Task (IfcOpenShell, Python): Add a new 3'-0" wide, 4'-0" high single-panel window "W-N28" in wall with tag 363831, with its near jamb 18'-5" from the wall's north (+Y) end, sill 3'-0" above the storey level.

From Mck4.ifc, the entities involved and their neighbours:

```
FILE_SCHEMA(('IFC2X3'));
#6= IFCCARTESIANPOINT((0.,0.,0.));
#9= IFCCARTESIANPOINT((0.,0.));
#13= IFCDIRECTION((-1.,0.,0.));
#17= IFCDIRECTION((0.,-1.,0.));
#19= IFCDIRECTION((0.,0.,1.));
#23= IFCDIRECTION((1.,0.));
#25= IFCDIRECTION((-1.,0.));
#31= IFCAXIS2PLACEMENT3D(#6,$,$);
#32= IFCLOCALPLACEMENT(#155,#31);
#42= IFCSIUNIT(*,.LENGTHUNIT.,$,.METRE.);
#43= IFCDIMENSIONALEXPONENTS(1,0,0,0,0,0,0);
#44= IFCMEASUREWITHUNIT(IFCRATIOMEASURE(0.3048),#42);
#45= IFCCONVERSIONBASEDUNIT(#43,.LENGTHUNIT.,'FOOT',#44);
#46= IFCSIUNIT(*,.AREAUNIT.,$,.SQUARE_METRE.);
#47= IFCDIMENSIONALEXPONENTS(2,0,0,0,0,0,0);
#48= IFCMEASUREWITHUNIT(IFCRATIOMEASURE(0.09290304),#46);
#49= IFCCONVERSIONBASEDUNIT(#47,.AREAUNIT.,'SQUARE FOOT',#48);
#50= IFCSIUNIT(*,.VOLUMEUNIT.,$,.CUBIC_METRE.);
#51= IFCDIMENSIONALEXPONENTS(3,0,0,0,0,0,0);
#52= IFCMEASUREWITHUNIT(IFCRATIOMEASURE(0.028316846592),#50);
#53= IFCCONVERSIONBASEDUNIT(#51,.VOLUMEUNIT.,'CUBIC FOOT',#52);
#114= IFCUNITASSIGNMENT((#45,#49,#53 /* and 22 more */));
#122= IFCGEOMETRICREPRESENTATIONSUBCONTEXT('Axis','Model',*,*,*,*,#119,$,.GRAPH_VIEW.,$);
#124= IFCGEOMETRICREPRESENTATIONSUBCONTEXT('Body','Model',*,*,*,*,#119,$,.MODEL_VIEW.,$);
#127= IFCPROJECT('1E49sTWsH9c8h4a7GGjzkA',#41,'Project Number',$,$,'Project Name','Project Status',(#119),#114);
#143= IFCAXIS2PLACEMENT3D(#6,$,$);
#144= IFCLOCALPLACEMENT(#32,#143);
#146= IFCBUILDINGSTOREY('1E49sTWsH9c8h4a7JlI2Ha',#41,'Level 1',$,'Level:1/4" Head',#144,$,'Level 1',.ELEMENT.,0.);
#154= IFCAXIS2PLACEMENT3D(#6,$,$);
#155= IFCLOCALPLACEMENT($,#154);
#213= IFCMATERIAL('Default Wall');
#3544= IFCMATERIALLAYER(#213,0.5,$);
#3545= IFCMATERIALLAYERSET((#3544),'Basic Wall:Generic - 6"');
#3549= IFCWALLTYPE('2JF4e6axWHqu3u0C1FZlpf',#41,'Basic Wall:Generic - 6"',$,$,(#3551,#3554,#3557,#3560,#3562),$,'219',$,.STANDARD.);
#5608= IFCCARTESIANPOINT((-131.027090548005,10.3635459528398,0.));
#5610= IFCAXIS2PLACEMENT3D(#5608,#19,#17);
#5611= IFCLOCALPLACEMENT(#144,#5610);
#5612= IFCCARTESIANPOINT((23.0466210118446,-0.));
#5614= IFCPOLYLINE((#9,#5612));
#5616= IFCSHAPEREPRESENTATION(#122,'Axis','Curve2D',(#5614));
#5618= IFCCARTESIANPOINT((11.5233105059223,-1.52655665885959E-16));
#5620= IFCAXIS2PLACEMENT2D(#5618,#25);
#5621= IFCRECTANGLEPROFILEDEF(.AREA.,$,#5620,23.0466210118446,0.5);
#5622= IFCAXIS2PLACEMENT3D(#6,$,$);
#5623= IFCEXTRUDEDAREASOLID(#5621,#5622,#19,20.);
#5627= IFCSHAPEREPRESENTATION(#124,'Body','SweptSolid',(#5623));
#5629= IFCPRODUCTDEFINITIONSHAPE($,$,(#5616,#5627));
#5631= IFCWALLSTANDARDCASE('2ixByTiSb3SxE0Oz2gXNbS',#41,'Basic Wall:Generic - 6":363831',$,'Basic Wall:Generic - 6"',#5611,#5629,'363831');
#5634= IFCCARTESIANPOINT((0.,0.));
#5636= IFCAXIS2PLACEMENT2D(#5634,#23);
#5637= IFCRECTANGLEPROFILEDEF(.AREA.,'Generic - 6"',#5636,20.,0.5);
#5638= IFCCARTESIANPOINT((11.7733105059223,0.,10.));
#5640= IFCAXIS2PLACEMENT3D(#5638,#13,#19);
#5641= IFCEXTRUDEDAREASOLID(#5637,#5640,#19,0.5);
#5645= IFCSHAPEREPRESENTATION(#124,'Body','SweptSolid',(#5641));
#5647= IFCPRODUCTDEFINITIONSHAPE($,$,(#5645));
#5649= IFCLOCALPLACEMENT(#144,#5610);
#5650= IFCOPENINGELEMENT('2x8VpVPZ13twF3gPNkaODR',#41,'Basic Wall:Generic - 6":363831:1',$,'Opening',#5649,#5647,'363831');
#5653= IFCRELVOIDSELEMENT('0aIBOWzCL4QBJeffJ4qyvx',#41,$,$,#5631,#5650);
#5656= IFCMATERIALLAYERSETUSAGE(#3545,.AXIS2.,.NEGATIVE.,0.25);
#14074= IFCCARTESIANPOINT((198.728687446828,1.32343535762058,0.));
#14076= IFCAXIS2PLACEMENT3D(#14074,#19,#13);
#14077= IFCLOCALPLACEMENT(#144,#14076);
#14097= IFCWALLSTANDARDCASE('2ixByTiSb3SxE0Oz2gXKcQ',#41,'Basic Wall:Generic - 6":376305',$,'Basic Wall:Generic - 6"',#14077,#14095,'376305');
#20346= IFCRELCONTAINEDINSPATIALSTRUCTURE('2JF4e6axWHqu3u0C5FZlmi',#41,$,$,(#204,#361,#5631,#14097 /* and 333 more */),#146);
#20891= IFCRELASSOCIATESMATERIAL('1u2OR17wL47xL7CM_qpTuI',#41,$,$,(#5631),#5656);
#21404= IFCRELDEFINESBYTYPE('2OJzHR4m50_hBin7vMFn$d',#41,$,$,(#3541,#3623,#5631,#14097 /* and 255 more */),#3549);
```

```python
import numpy as np
import ifcopenshell
import ifcopenshell.api.feature
import ifcopenshell.api.geometry
import ifcopenshell.api.root
import ifcopenshell.api.spatial
import ifcopenshell.api.type
import ifcopenshell.geom
import ifcopenshell.util.element
import ifcopenshell.util.placement
import ifcopenshell.util.representation
import ifcopenshell.util.shape
import ifcopenshell.util.unit

model = ifcopenshell.open("Mck4.ifc")
unit_scale = ifcopenshell.util.unit.calculate_unit_scale(model)
settings = ifcopenshell.geom.settings()


def volume(element):
    """Net volume in cubic metres, openings subtracted."""
    shape = ifcopenshell.geom.create_shape(settings, element)
    return ifcopenshell.util.shape.get_volume(shape.geometry)


wall = model.by_id(5631)
storey = ifcopenshell.util.element.get_container(wall, ifc_class="IfcBuildingStorey")
context = ifcopenshell.util.representation.get_context(model, "Model", "Body", "MODEL_VIEW")
before = volume(wall)

width, height, from_end, sill = 0.9144, 1.2192, 5.6134, 0.9144  # metres

# The wall runs along its own X axis, and the end named is its -X end.
wall_shape = ifcopenshell.geom.create_shape(settings, wall)
x, y, z = ifcopenshell.util.shape.get_vertices(wall_shape.geometry).T
start = x.min() + from_end
face, thickness = float(y.min()), float(y.max() - y.min())
wall_matrix = ifcopenshell.util.placement.get_local_placement(wall.ObjectPlacement)
level = ifcopenshell.util.placement.get_local_placement(storey.ObjectPlacement)[2, 3]


def in_wall(x, y):
    """Placement at x, y metres in the wall's axes, at sill height."""
    matrix = wall_matrix.copy()
    matrix[:, 3] = wall_matrix @ np.array([x / unit_scale, y / unit_scale, 0.0, 1.0])
    matrix[2, 3] = level + sill / unit_scale
    return matrix


# Opening: a box that overshoots both wall faces by 50 mm.
opening = ifcopenshell.api.root.create_entity(model, ifc_class="IfcOpeningElement")
box = ifcopenshell.api.geometry.add_wall_representation(
    model, context=context, length=width, height=height, thickness=thickness + 0.1
)
ifcopenshell.api.geometry.assign_representation(model, product=opening, representation=box)
ifcopenshell.api.geometry.edit_object_placement(model, product=opening, matrix=in_wall(start, face - 0.05), is_si=False)
ifcopenshell.api.feature.add_feature(model, feature=opening, element=wall)

window = ifcopenshell.api.root.create_entity(model, ifc_class="IfcWindow", name="W-N28")
window.OverallWidth, window.OverallHeight = width / unit_scale, height / unit_scale
body = ifcopenshell.api.geometry.add_window_representation(
    model,
    context=context,
    overall_width=window.OverallWidth,
    overall_height=window.OverallHeight,
    partition_type="SINGLE_PANEL",
)
ifcopenshell.api.geometry.assign_representation(model, product=window, representation=body)
ifcopenshell.api.spatial.assign_container(model, products=[window], relating_structure=storey)
fills = ifcopenshell.api.feature.add_filling(model, opening=opening, element=window)
fills.OwnerHistory = window.OwnerHistory  # required in IFC2X3

# IFC2X3 keeps the operation on the window style.
style = ifcopenshell.api.root.create_entity(model, ifc_class="IfcWindowStyle", name="W-N28")
style.OperationType, style.ConstructionType = "SINGLE_PANEL", "NOTDEFINED"
style.ParameterTakesPrecedence = style.Sizeable = False
ifcopenshell.api.type.assign_type(model, related_objects=[window], relating_type=style)

# Centre the window in the wall's thickness.
ifcopenshell.api.geometry.edit_object_placement(model, product=window, matrix=in_wall(start, face), is_si=False)
window_shape = ifcopenshell.geom.create_shape(settings, window)
depth = ifcopenshell.util.shape.get_vertices(window_shape.geometry)[:, 1]
offset = face + thickness / 2 - (depth.min() + depth.max()) / 2
ifcopenshell.api.geometry.edit_object_placement(model, product=window, matrix=in_wall(start, offset), is_si=False)

after = volume(wall)

print(f"wall volume {before:.3f} -> {after:.3f} m3")

model.write("Mck4_updated.ifc")
```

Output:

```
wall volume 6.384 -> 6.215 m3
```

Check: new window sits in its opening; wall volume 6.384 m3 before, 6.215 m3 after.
